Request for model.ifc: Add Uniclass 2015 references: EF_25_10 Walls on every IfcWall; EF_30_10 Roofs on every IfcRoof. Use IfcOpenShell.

First a look at what the model holds.

```python
import ifcopenshell

model = ifcopenshell.open("model.ifc")
print(model.schema)
print("classifications:", [c.Name for c in model.by_type("IfcClassification")])
for ifc_class in ("IfcDoor", "IfcRoof", "IfcStair", "IfcWall", "IfcWindow"):
    print(ifc_class, len(model.by_type(ifc_class)))
```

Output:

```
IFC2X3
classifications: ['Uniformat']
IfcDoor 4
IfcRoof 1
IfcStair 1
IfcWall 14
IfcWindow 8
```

```python
import ifcopenshell
import ifcopenshell.api.classification

model = ifcopenshell.open("model.ifc")

# IFC2X3 requires Source and Edition and has no link from the project to the system.
system = model.create_entity("IfcClassification", Source="NBS", Edition="2015", Name="Uniclass 2015")

codes = {
    "IfcWall": ("EF_25_10", "Walls"),
    "IfcRoof": ("EF_30_10", "Roofs"),
}
for ifc_class, (code, name) in codes.items():
    products = model.by_type(ifc_class)
    ifcopenshell.api.classification.add_reference(
        model, products=products, classification=system, identification=code, name=name
    )
    print(code, len(products))

model.write("model_updated.ifc")
```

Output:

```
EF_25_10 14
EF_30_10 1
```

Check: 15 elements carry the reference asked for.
